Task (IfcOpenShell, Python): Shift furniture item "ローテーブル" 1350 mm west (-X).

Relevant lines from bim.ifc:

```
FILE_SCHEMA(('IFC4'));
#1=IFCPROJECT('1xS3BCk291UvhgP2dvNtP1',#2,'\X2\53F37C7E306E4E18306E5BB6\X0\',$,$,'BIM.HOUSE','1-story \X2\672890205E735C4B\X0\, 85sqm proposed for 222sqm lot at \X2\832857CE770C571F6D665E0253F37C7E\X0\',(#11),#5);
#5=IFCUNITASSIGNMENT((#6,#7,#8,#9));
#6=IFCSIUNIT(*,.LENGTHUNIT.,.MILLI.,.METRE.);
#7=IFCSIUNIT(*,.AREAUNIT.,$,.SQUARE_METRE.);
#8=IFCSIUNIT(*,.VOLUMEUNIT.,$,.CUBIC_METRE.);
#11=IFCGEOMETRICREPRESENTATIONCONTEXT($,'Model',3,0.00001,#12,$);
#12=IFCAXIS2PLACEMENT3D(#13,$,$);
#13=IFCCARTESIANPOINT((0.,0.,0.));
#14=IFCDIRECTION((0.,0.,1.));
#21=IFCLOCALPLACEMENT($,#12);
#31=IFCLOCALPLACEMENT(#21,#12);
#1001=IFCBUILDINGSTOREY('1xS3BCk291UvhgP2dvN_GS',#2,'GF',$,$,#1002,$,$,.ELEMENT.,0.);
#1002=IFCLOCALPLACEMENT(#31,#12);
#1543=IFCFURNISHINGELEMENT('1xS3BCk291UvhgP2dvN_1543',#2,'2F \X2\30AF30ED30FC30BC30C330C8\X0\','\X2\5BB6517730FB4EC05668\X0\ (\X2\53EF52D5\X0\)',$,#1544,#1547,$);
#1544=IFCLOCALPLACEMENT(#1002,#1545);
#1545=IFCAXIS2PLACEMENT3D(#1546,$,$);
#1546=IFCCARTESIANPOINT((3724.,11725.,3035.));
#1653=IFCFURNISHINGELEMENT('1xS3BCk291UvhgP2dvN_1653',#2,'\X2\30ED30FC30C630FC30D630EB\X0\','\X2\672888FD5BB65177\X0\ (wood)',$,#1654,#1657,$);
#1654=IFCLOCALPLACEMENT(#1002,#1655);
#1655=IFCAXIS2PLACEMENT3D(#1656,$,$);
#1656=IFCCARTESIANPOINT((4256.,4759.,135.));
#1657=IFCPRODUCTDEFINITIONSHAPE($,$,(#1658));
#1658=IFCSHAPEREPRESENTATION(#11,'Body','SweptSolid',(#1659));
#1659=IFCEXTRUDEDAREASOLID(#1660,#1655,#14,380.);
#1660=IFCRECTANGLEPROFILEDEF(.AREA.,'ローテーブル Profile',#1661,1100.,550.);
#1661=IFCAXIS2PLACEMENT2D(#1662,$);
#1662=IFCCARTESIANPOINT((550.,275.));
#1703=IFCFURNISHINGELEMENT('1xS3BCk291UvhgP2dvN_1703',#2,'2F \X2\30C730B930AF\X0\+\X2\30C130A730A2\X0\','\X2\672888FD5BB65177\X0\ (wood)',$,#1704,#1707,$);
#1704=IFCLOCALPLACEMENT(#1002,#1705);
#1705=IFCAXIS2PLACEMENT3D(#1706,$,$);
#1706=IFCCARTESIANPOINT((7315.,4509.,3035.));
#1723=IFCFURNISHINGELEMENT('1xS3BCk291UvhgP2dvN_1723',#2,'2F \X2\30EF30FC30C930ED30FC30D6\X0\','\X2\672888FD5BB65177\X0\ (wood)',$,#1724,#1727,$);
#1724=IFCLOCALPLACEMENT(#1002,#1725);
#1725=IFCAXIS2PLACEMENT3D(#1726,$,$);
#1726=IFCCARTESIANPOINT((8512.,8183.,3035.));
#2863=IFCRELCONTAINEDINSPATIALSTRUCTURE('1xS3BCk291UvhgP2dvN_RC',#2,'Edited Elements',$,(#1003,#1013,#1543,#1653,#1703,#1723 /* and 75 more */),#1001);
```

```python
import ifcopenshell
import ifcopenshell.api.geometry
import ifcopenshell.util.placement
import ifcopenshell.util.unit

model = ifcopenshell.open("bim.ifc")
unit_scale = ifcopenshell.util.unit.calculate_unit_scale(model)

item = model.by_id(1653)
matrix = ifcopenshell.util.placement.get_local_placement(item.ObjectPlacement)
matrix[0, 3] -= 1.35 / unit_scale
ifcopenshell.api.geometry.edit_object_placement(model, product=item, matrix=matrix, is_si=False)

print(ifcopenshell.util.placement.get_local_placement(item.ObjectPlacement).round(3) + 0.0)

model.write("bim_updated.ifc")
```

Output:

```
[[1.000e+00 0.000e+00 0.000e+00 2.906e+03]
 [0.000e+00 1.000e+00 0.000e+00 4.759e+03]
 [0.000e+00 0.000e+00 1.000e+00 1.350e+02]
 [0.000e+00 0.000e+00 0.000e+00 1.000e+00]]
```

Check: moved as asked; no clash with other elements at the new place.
